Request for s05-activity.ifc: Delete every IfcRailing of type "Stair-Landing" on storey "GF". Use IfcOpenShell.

First a look at what the model holds.

```python
import ifcopenshell
import ifcopenshell.util.element

model = ifcopenshell.open("s05-activity.ifc")
print(model.schema)
storey = next(s for s in model.by_type("IfcBuildingStorey") if s.Name == "GF")
railings = [e for e in ifcopenshell.util.element.get_decomposition(storey) if e.is_a("IfcRailing")]
seen = {}
for e in railings:
    element_type = ifcopenshell.util.element.get_type(e)
    name = element_type.Name if element_type not in (None, e) else None
    seen[name] = seen.get(name, 0) + 1
for name, count in sorted(seen.items(), key=str):
    print(count, "x", name)
```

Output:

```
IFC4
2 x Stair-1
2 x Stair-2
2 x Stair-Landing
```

```python
import ifcopenshell
import ifcopenshell.api.root
import ifcopenshell.util.element

model = ifcopenshell.open("s05-activity.ifc")

storey = next(s for s in model.by_type("IfcBuildingStorey") if s.Name == "GF")
railings = [e for e in ifcopenshell.util.element.get_decomposition(storey) if e.is_a("IfcRailing")]
targets = [e for e in railings if (t := ifcopenshell.util.element.get_type(e)) not in (None, e) and t.Name == "Stair-Landing"]

for e in targets:
    ifcopenshell.api.root.remove_product(model, product=e)
print(len(targets), "removed")

model.write("s05-activity_v2.ifc")
```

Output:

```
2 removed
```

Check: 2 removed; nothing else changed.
